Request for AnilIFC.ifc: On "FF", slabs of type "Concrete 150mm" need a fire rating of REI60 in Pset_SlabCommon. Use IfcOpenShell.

First a look at what the model holds.

```python
import ifcopenshell
import ifcopenshell.util.element

model = ifcopenshell.open("AnilIFC.ifc")
print(model.schema)
storey = next(s for s in model.by_type("IfcBuildingStorey") if s.Name == "FF")
slabs = [e for e in ifcopenshell.util.element.get_decomposition(storey) if e.is_a("IfcSlab")]
seen = {}
for e in slabs:
    element_type = ifcopenshell.util.element.get_type(e)
    key = (element_type.Name if element_type != e and element_type else None, ifcopenshell.util.element.get_pset(e, "Pset_SlabCommon", "FireRating"))
    seen[key] = seen.get(key, 0) + 1
for (name, value), count in sorted(seen.items(), key=str):
    print(count, "x", name, "|", value)
```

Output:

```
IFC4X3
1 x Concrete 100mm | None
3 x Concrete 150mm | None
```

```python
import ifcopenshell
import ifcopenshell.api.pset
import ifcopenshell.util.element

model = ifcopenshell.open("AnilIFC.ifc")

storey = next(s for s in model.by_type("IfcBuildingStorey") if s.Name == "FF")
slabs = [e for e in ifcopenshell.util.element.get_decomposition(storey) if e.is_a("IfcSlab")]

count = 0
for e in slabs:
    element_type = ifcopenshell.util.element.get_type(e)
    if element_type in (None, e) or element_type.Name != "Concrete 150mm":
        continue
    # add_pset returns the element's existing set when there is one.
    pset = ifcopenshell.api.pset.add_pset(model, product=e, name="Pset_SlabCommon")
    ifcopenshell.api.pset.edit_pset(model, pset=pset, properties={"FireRating": "REI60"})
    count += 1

print(count, "slabs updated")

model.write("AnilIFC_updated.ifc")
```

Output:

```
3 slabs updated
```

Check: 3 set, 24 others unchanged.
